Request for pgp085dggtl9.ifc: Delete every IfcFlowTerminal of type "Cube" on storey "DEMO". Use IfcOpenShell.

First a look at what the model holds.

```python
import ifcopenshell
import ifcopenshell.util.element

model = ifcopenshell.open("pgp085dggtl9.ifc")
print(model.schema)
storey = next(s for s in model.by_type("IfcBuildingStorey") if s.Name == "DEMO")
terminals = [e for e in ifcopenshell.util.element.get_decomposition(storey) if e.is_a("IfcFlowTerminal")]
seen = {}
for e in terminals:
    element_type = ifcopenshell.util.element.get_type(e)
    name = element_type.Name if element_type not in (None, e) else None
    seen[name] = seen.get(name, 0) + 1
for name, count in sorted(seen.items(), key=str):
    print(count, "x", name)
```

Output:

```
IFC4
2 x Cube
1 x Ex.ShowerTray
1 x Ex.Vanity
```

```python
import ifcopenshell
import ifcopenshell.api.root
import ifcopenshell.util.element

model = ifcopenshell.open("pgp085dggtl9.ifc")

storey = next(s for s in model.by_type("IfcBuildingStorey") if s.Name == "DEMO")
terminals = [e for e in ifcopenshell.util.element.get_decomposition(storey) if e.is_a("IfcFlowTerminal")]
targets = [e for e in terminals if (t := ifcopenshell.util.element.get_type(e)) not in (None, e) and t.Name == "Cube"]

for e in targets:
    ifcopenshell.api.root.remove_product(model, product=e)
print(len(targets), "removed")

model.write("pgp085dggtl9_edited.ifc")
```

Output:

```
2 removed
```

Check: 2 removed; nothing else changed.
